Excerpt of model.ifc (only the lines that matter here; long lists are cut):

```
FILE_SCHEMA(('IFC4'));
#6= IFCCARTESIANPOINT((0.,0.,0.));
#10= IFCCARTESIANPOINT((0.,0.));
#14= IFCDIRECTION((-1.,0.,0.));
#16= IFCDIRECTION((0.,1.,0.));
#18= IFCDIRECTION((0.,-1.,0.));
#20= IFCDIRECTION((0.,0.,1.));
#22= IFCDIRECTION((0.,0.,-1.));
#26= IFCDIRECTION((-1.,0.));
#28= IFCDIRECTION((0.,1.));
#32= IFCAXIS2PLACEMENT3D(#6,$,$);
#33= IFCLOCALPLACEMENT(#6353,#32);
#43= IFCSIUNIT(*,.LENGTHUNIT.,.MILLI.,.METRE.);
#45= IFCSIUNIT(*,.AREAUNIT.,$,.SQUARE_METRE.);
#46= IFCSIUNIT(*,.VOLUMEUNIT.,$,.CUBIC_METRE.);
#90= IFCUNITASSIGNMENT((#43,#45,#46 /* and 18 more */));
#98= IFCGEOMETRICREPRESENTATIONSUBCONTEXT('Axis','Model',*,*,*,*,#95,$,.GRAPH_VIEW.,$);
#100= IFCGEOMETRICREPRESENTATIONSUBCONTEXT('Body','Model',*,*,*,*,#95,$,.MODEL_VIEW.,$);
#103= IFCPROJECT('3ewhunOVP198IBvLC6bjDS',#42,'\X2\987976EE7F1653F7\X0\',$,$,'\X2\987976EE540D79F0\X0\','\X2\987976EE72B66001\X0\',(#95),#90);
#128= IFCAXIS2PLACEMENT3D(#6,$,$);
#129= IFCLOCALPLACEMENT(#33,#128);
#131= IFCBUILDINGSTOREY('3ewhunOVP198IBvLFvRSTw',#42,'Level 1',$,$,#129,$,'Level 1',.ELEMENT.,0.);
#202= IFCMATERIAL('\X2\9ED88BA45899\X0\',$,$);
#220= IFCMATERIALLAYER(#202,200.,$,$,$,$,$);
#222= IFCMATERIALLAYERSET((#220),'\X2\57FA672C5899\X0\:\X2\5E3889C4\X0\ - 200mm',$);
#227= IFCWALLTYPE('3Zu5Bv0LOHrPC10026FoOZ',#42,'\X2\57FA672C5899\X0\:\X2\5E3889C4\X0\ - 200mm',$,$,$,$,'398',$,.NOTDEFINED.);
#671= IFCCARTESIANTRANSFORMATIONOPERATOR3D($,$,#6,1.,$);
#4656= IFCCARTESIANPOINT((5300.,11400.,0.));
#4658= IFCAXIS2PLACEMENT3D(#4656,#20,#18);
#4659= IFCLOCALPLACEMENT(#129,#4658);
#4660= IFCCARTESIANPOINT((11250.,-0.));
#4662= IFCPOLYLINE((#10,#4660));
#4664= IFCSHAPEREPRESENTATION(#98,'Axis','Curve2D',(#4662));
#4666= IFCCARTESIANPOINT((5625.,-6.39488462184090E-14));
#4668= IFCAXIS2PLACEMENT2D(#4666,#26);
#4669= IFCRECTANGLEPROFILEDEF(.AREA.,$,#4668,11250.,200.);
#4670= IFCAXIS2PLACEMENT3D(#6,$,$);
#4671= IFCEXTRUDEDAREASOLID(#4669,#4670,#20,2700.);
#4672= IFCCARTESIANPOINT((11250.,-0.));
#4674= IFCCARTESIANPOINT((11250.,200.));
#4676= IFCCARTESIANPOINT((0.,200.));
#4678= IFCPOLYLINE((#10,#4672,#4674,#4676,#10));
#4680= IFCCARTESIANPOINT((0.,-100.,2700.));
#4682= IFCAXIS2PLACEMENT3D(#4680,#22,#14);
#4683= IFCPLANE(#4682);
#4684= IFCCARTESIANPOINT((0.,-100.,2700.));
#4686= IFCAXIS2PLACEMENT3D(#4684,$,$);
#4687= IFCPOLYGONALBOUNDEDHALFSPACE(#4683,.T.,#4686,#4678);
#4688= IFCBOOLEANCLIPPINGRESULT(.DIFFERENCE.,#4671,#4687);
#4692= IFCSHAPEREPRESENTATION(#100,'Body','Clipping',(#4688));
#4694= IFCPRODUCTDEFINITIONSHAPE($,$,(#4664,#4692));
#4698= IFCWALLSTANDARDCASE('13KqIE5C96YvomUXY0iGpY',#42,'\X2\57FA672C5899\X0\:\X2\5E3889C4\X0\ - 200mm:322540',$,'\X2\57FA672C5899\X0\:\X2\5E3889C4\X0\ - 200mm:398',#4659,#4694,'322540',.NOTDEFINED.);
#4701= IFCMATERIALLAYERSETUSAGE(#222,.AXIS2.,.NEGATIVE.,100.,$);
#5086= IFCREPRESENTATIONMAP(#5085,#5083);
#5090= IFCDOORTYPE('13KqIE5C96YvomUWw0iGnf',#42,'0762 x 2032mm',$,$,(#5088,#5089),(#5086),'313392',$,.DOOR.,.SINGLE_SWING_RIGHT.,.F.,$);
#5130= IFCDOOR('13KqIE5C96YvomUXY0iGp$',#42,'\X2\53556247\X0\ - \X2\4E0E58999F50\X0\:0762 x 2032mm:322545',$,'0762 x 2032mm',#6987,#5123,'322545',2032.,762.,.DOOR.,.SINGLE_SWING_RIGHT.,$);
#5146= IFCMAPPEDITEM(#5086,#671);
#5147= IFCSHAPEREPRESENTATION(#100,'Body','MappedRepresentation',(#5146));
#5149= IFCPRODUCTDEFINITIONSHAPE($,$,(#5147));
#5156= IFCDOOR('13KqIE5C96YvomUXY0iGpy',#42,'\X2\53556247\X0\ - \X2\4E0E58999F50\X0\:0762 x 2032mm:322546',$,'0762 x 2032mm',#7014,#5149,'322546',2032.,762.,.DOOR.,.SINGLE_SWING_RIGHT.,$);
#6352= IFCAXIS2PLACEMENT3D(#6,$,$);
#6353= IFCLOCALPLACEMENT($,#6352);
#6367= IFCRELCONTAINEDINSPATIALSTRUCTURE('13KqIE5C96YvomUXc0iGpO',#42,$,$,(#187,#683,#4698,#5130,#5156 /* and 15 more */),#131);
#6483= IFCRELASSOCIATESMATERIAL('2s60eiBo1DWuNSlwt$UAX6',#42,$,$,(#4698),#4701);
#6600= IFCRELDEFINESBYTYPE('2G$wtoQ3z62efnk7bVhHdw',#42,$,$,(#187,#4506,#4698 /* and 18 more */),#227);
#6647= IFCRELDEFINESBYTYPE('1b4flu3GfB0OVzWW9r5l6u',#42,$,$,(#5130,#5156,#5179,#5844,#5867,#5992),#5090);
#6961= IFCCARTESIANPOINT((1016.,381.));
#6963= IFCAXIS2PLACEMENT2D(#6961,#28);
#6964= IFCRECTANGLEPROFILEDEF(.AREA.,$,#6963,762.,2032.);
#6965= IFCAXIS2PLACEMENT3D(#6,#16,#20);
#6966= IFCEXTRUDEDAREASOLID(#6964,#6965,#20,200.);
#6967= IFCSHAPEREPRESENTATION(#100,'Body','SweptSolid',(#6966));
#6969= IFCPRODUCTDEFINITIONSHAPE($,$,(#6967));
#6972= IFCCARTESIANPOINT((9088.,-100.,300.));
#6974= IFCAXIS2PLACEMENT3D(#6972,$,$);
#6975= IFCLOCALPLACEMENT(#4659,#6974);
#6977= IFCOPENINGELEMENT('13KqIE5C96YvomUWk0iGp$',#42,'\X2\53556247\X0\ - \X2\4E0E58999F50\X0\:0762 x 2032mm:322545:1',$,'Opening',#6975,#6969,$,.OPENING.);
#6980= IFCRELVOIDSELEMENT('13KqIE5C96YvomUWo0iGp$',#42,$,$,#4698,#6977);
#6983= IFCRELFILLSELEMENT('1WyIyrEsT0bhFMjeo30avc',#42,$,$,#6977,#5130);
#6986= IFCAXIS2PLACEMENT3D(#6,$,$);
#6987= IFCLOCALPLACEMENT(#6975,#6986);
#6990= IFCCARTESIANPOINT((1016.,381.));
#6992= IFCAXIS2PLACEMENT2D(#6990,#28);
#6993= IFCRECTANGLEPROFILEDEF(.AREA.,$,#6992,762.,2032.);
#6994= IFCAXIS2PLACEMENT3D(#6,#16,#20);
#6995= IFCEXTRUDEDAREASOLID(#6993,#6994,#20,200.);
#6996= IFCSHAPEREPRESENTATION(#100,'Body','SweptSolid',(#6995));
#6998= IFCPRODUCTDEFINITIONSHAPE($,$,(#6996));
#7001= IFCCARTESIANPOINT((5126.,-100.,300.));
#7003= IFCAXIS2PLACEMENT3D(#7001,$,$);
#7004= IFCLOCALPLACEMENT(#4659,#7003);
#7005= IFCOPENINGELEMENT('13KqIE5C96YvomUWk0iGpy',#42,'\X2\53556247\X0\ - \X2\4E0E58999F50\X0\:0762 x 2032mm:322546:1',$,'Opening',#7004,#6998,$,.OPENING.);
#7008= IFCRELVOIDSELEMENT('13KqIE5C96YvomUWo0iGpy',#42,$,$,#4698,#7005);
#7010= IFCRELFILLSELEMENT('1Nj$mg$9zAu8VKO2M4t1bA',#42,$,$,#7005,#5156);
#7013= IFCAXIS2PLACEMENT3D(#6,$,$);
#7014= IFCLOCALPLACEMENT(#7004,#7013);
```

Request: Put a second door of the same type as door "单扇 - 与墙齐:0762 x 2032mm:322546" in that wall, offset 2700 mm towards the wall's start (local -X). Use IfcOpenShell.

```python
import ifcopenshell
import ifcopenshell.api.feature
import ifcopenshell.api.geometry
import ifcopenshell.api.root
import ifcopenshell.geom
import ifcopenshell.util.element
import ifcopenshell.util.placement
import ifcopenshell.util.shape

model = ifcopenshell.open("model.ifc")
settings = ifcopenshell.geom.settings()


def volume(element):
    """Net volume in cubic metres, openings subtracted."""
    shape = ifcopenshell.geom.create_shape(settings, element)
    return ifcopenshell.util.shape.get_volume(shape.geometry)


def reuse_history(source, copy):
    """copy_class also copies each property set's owner history, people and application; keep the originals."""
    for rel in copy.IsDefinedBy:
        if rel.is_a("IfcRelDefinesByProperties") and (history := rel.RelatingPropertyDefinition.OwnerHistory):
            rel.RelatingPropertyDefinition.OwnerHistory = source.OwnerHistory
            ifcopenshell.util.element.remove_deep2(model, history)


door = model.by_id(5156)
opening = door.FillsVoids[0].RelatingOpeningElement
wall = opening.VoidsElements[0].RelatingBuildingElement
before = volume(wall)
shift = ifcopenshell.util.placement.get_local_placement(wall.ObjectPlacement)[:3, 0] * -2700.0

# copy_class copies the void relationship, type, container and properties, but no geometry.
new_opening = ifcopenshell.api.root.copy_class(model, product=opening)
new_opening.Representation = ifcopenshell.util.element.copy_deep(
    model, opening.Representation, exclude=["IfcGeometricRepresentationContext", "IfcRepresentationMap"]
)
new_opening.Name = "单扇 - 与墙齐:0762 x 2032mm"
new_door = ifcopenshell.api.root.copy_class(model, product=door)
new_door.Representation = ifcopenshell.util.element.copy_deep(
    model, door.Representation, exclude=["IfcGeometricRepresentationContext", "IfcRepresentationMap"]
)
new_door.Name = "单扇 - 与墙齐:0762 x 2032mm"
new_door.Tag = None
reuse_history(door, new_door)
ifcopenshell.api.feature.add_filling(model, opening=new_opening, element=new_door)

for old, new in ((opening, new_opening), (door, new_door)):
    matrix = ifcopenshell.util.placement.get_local_placement(old.ObjectPlacement)
    matrix[:3, 3] += shift
    ifcopenshell.api.geometry.edit_object_placement(model, product=new, matrix=matrix, is_si=False)

after = volume(wall)

print(f"wall volume {before:.3f} -> {after:.3f} m3")

model.write("model_rev.ifc")
```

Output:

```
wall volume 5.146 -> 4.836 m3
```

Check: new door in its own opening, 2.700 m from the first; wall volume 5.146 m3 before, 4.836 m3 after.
